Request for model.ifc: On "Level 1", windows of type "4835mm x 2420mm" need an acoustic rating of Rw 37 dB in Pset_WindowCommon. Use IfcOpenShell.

First a look at what the model holds.

```python
import ifcopenshell
import ifcopenshell.util.element

model = ifcopenshell.open("model.ifc")
print(model.schema)
storey = next(s for s in model.by_type("IfcBuildingStorey") if s.Name == "Level 1")
windows = [e for e in ifcopenshell.util.element.get_decomposition(storey) if e.is_a("IfcWindow")]
seen = {}
for e in windows:
    element_type = ifcopenshell.util.element.get_type(e)
    key = (element_type.Name if element_type != e and element_type else None, ifcopenshell.util.element.get_pset(e, "Pset_WindowCommon", "AcousticRating"))
    seen[key] = seen.get(key, 0) + 1
for (name, value), count in sorted(seen.items(), key=str):
    print(count, "x", name, "|", value)
```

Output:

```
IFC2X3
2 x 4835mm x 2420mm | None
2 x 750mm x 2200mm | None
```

```python
import ifcopenshell
import ifcopenshell.api.pset
import ifcopenshell.util.element

model = ifcopenshell.open("model.ifc")

storey = next(s for s in model.by_type("IfcBuildingStorey") if s.Name == "Level 1")
windows = [e for e in ifcopenshell.util.element.get_decomposition(storey) if e.is_a("IfcWindow")]

count = 0
for e in windows:
    element_type = ifcopenshell.util.element.get_type(e)
    if element_type in (None, e) or element_type.Name != "4835mm x 2420mm":
        continue
    # add_pset returns the element's existing set when there is one.
    pset = ifcopenshell.api.pset.add_pset(model, product=e, name="Pset_WindowCommon")
    ifcopenshell.api.pset.edit_pset(model, pset=pset, properties={"AcousticRating": "Rw 37 dB"})
    count += 1

print(count, "windows updated")

model.write("model_edited.ifc")
```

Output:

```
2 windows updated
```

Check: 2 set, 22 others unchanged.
